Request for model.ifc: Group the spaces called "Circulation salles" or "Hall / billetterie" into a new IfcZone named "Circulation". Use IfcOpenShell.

First a look at what the model holds.

```python
import ifcopenshell

model = ifcopenshell.open("model.ifc")
print(model.schema)
seen = {}
for space in model.by_type("IfcSpace"):
    seen[space.LongName] = seen.get(space.LongName, 0) + 1
for name, count in sorted(seen.items(), key=str):
    print(count, "x", name)
print("zones:", [z.Name for z in model.by_type("IfcZone")][:20])
```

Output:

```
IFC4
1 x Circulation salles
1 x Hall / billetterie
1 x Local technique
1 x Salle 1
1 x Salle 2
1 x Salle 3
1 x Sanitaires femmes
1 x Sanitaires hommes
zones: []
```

```python
import ifcopenshell
import ifcopenshell.api.group
import ifcopenshell.api.root

model = ifcopenshell.open("model.ifc")

names = {"Circulation salles", "Hall / billetterie"}
spaces = [s for s in model.by_type("IfcSpace") if s.LongName in names]

zone = ifcopenshell.api.root.create_entity(model, ifc_class="IfcZone", name="Circulation")
ifcopenshell.api.group.assign_group(model, products=spaces, group=zone)
print(len(spaces), "spaces in", zone.Name)

model.write("model_updated.ifc")
```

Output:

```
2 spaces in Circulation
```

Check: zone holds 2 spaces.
